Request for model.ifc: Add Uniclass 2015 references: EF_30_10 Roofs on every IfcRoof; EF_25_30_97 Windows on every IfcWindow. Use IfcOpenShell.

First a look at what the model holds.

```python
import ifcopenshell

model = ifcopenshell.open("model.ifc")
print(model.schema)
print("classifications:", [c.Name for c in model.by_type("IfcClassification")])
for ifc_class in ("IfcDoor", "IfcRoof", "IfcStair", "IfcWall", "IfcWindow"):
    print(ifc_class, len(model.by_type(ifc_class)))
```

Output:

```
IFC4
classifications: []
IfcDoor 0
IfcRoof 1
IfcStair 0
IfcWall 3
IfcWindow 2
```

```python
import ifcopenshell
import ifcopenshell.api.classification

model = ifcopenshell.open("model.ifc")

system = ifcopenshell.api.classification.add_classification(model, classification="Uniclass 2015")

codes = {
    "IfcRoof": ("EF_30_10", "Roofs"),
    "IfcWindow": ("EF_25_30_97", "Windows"),
}
for ifc_class, (code, name) in codes.items():
    products = model.by_type(ifc_class)
    ifcopenshell.api.classification.add_reference(
        model, products=products, classification=system, identification=code, name=name
    )
    print(code, len(products))

model.write("model-out.ifc")
```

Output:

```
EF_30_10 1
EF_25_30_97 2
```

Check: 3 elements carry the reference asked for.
